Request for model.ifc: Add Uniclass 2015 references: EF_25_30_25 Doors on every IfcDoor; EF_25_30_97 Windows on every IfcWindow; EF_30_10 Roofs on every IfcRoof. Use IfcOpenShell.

First a look at what the model holds.

```python
import ifcopenshell

model = ifcopenshell.open("model.ifc")
print(model.schema)
print("classifications:", [c.Name for c in model.by_type("IfcClassification")])
for ifc_class in ("IfcDoor", "IfcRoof", "IfcStair", "IfcWall", "IfcWindow"):
    print(ifc_class, len(model.by_type(ifc_class)))
```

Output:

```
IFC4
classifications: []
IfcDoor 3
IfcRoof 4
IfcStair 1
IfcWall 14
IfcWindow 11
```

```python
import ifcopenshell
import ifcopenshell.api.classification

model = ifcopenshell.open("model.ifc")

system = ifcopenshell.api.classification.add_classification(model, classification="Uniclass 2015")

codes = {
    "IfcDoor": ("EF_25_30_25", "Doors"),
    "IfcWindow": ("EF_25_30_97", "Windows"),
    "IfcRoof": ("EF_30_10", "Roofs"),
}
for ifc_class, (code, name) in codes.items():
    products = model.by_type(ifc_class)
    ifcopenshell.api.classification.add_reference(
        model, products=products, classification=system, identification=code, name=name
    )
    print(code, len(products))

model.write("model_updated.ifc")
```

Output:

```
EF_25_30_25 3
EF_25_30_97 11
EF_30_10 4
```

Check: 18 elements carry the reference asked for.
